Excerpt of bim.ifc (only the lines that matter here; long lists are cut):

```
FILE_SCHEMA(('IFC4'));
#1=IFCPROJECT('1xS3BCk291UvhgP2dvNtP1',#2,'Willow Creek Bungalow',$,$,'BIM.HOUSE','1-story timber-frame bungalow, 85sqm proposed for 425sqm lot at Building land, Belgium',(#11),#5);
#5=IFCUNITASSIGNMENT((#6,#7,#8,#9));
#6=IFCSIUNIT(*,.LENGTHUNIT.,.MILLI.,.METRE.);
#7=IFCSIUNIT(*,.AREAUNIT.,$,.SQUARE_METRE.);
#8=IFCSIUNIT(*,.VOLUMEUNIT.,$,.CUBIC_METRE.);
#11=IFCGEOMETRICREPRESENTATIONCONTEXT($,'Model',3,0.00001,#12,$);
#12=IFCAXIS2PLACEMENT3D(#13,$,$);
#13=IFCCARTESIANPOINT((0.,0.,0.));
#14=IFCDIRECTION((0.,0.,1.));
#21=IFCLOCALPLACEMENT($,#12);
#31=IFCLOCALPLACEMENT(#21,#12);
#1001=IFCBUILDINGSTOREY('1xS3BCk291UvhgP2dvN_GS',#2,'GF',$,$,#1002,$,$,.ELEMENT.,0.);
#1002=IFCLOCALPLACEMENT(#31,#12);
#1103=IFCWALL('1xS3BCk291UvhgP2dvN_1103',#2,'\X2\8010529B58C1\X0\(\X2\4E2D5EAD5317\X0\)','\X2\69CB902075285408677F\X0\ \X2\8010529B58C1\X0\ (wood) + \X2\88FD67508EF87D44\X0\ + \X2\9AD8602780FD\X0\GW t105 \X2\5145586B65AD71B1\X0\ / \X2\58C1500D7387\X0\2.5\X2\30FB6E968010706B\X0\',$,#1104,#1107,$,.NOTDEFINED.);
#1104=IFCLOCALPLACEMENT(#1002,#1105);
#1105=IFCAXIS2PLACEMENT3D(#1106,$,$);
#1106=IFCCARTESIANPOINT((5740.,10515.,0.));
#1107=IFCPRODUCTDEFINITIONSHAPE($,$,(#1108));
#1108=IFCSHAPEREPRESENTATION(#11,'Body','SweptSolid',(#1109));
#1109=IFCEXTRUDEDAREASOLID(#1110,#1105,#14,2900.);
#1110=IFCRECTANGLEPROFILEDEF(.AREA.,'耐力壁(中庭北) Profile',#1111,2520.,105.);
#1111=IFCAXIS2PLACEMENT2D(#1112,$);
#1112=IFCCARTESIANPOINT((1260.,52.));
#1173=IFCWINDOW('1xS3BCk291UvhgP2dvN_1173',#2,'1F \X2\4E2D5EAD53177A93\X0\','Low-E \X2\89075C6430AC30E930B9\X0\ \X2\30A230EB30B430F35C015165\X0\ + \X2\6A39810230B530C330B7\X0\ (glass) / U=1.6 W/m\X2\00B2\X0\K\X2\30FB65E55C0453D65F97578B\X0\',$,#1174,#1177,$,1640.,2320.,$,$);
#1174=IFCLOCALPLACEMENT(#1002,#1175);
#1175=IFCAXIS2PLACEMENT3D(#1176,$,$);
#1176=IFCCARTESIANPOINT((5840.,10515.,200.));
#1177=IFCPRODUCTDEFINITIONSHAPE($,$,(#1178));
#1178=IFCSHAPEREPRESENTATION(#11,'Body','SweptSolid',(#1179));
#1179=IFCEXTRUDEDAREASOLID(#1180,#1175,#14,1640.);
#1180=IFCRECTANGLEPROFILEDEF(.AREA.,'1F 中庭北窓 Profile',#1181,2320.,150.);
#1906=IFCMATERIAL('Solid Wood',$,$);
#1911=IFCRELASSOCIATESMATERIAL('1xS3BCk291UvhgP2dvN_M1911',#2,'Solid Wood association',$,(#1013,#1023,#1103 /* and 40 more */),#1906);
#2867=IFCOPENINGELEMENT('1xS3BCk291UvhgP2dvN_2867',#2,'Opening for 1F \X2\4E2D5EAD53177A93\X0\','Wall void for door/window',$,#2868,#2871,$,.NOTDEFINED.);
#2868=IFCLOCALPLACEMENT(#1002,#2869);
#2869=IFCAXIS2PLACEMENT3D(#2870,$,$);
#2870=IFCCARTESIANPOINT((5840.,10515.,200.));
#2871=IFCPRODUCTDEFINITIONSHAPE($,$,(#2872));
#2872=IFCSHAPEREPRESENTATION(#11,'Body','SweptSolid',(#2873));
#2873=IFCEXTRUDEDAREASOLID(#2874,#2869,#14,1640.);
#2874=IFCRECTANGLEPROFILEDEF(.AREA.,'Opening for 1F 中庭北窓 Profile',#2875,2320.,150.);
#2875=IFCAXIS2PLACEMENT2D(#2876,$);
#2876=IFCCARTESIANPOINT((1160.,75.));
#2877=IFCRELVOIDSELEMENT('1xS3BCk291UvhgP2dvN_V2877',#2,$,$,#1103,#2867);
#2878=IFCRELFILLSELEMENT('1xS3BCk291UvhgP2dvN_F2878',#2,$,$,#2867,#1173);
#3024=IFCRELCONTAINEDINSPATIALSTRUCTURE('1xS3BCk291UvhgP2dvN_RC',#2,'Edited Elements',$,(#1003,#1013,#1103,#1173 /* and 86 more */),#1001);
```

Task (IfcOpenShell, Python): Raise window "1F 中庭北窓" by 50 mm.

```python
import numpy as np
import ifcopenshell
import ifcopenshell.api.geometry
import ifcopenshell.util.placement
import ifcopenshell.util.unit

model = ifcopenshell.open("bim.ifc")
unit_scale = ifcopenshell.util.unit.calculate_unit_scale(model)

window = model.by_guid("1xS3BCk291UvhgP2dvN_1173")
opening = window.FillsVoids[0].RelatingOpeningElement
dz = 0.05 / unit_scale

shift = np.array([0.0, 0.0, dz])
# The window is not placed relative to its opening, so move both.
for product in (opening, window):
    matrix = ifcopenshell.util.placement.get_local_placement(product.ObjectPlacement)
    matrix[:3, 3] += shift
    ifcopenshell.api.geometry.edit_object_placement(model, product=product, matrix=matrix, is_si=False)

print(f"moved by {dz * unit_scale:+.3f} m")

model.write("bim-out.ifc")
```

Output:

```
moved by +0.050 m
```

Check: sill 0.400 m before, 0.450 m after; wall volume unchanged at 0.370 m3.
